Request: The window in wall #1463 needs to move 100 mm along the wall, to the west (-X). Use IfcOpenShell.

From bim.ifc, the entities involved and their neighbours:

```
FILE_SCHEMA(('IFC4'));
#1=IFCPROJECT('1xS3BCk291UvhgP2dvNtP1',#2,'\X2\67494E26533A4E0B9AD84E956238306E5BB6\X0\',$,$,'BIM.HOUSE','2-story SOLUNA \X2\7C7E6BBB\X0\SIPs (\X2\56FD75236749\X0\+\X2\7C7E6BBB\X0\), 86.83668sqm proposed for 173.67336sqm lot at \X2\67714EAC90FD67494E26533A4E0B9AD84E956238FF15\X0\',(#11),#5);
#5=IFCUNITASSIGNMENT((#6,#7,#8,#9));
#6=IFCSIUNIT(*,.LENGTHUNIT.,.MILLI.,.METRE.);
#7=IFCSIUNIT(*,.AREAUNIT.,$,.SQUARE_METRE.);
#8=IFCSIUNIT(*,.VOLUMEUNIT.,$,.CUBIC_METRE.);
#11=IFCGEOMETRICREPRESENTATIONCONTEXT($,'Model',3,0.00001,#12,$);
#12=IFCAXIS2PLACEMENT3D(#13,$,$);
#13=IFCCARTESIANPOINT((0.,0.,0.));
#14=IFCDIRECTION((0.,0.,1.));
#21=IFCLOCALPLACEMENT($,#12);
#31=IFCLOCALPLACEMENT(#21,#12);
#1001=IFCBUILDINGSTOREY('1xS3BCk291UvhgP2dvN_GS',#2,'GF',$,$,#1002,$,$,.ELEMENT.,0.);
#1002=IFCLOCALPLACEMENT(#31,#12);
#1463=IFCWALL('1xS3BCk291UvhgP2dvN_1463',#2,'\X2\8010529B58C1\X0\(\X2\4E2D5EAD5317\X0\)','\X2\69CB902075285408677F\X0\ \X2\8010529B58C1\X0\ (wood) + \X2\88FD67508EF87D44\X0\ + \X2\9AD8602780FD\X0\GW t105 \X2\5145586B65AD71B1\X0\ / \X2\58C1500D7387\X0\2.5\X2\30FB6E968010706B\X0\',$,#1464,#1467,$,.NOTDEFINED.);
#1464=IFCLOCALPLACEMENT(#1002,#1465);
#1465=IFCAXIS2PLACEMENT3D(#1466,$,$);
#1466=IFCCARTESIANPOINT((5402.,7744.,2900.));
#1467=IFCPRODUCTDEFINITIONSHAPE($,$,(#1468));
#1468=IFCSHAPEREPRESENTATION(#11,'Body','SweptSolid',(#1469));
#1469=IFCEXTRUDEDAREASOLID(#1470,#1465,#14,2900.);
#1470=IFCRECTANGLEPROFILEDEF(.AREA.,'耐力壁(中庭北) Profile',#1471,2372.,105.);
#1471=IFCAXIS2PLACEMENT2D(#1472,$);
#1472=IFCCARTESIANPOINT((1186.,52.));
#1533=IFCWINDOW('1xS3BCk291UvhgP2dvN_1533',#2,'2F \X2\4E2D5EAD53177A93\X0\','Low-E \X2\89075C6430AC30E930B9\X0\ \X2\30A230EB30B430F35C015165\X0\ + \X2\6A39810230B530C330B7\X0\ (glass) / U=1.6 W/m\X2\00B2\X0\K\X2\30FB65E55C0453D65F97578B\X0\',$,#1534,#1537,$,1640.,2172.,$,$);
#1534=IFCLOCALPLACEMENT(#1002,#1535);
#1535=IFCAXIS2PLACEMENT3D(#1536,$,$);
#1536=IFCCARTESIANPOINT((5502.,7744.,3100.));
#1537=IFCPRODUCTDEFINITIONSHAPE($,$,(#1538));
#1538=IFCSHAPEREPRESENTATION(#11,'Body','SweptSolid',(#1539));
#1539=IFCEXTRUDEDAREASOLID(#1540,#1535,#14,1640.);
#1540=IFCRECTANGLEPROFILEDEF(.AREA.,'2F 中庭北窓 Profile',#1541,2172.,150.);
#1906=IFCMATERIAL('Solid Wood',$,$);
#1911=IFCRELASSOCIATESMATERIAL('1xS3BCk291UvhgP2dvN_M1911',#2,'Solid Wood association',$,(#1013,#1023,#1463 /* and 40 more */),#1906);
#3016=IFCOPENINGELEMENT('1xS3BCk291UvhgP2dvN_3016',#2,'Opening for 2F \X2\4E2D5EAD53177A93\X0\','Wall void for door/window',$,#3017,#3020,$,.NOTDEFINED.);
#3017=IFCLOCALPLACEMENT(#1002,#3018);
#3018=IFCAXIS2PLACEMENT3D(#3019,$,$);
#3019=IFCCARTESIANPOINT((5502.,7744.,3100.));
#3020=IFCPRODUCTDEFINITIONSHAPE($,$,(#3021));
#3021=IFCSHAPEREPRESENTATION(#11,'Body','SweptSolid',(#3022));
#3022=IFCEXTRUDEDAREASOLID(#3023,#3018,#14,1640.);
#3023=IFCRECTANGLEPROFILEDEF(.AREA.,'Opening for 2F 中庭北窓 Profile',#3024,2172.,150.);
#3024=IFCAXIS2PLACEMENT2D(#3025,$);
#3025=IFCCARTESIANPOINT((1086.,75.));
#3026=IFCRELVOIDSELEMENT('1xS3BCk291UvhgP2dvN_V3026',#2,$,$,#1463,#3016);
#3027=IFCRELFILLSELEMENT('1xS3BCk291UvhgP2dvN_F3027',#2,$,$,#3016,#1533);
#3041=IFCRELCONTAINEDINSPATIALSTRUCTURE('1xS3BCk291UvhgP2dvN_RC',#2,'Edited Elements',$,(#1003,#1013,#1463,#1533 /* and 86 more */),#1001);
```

```python
import ifcopenshell
import ifcopenshell.api.geometry
import ifcopenshell.util.placement

model = ifcopenshell.open("bim.ifc")

window = model.by_id(1533)
opening = window.FillsVoids[0].RelatingOpeningElement
wall = opening.VoidsElements[0].RelatingBuildingElement

wall_matrix = ifcopenshell.util.placement.get_local_placement(wall.ObjectPlacement)
shift = wall_matrix[:3, 0] * -100.0
before = ifcopenshell.util.placement.get_local_placement(window.ObjectPlacement)[:3, 3].copy()

# The window is not placed relative to its opening, so move both.
for product in (opening, window):
    matrix = ifcopenshell.util.placement.get_local_placement(product.ObjectPlacement)
    matrix[:3, 3] += shift
    ifcopenshell.api.geometry.edit_object_placement(model, product=product, matrix=matrix, is_si=False)

after = ifcopenshell.util.placement.get_local_placement(window.ObjectPlacement)[:3, 3]
print("window moved by", (after - before).round(3) + 0.0)

model.write("bim_rev.ifc")
```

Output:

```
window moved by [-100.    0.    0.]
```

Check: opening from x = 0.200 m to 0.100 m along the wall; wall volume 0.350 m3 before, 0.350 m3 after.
